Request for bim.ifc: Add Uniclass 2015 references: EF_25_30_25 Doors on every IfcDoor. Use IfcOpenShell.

First a look at what the model holds.

```python
import ifcopenshell

model = ifcopenshell.open("bim.ifc")
print(model.schema)
print("classifications:", [c.Name for c in model.by_type("IfcClassification")])
for ifc_class in ("IfcDoor", "IfcRoof", "IfcStair", "IfcWall", "IfcWindow"):
    print(ifc_class, len(model.by_type(ifc_class)))
```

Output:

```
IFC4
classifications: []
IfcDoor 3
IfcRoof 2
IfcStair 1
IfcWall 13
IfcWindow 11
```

```python
import ifcopenshell
import ifcopenshell.api.classification

model = ifcopenshell.open("bim.ifc")

system = ifcopenshell.api.classification.add_classification(model, classification="Uniclass 2015")

codes = {
    "IfcDoor": ("EF_25_30_25", "Doors"),
}
for ifc_class, (code, name) in codes.items():
    products = model.by_type(ifc_class)
    ifcopenshell.api.classification.add_reference(
        model, products=products, classification=system, identification=code, name=name
    )
    print(code, len(products))

model.write("bim-out.ifc")
```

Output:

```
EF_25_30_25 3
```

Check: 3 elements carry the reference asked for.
